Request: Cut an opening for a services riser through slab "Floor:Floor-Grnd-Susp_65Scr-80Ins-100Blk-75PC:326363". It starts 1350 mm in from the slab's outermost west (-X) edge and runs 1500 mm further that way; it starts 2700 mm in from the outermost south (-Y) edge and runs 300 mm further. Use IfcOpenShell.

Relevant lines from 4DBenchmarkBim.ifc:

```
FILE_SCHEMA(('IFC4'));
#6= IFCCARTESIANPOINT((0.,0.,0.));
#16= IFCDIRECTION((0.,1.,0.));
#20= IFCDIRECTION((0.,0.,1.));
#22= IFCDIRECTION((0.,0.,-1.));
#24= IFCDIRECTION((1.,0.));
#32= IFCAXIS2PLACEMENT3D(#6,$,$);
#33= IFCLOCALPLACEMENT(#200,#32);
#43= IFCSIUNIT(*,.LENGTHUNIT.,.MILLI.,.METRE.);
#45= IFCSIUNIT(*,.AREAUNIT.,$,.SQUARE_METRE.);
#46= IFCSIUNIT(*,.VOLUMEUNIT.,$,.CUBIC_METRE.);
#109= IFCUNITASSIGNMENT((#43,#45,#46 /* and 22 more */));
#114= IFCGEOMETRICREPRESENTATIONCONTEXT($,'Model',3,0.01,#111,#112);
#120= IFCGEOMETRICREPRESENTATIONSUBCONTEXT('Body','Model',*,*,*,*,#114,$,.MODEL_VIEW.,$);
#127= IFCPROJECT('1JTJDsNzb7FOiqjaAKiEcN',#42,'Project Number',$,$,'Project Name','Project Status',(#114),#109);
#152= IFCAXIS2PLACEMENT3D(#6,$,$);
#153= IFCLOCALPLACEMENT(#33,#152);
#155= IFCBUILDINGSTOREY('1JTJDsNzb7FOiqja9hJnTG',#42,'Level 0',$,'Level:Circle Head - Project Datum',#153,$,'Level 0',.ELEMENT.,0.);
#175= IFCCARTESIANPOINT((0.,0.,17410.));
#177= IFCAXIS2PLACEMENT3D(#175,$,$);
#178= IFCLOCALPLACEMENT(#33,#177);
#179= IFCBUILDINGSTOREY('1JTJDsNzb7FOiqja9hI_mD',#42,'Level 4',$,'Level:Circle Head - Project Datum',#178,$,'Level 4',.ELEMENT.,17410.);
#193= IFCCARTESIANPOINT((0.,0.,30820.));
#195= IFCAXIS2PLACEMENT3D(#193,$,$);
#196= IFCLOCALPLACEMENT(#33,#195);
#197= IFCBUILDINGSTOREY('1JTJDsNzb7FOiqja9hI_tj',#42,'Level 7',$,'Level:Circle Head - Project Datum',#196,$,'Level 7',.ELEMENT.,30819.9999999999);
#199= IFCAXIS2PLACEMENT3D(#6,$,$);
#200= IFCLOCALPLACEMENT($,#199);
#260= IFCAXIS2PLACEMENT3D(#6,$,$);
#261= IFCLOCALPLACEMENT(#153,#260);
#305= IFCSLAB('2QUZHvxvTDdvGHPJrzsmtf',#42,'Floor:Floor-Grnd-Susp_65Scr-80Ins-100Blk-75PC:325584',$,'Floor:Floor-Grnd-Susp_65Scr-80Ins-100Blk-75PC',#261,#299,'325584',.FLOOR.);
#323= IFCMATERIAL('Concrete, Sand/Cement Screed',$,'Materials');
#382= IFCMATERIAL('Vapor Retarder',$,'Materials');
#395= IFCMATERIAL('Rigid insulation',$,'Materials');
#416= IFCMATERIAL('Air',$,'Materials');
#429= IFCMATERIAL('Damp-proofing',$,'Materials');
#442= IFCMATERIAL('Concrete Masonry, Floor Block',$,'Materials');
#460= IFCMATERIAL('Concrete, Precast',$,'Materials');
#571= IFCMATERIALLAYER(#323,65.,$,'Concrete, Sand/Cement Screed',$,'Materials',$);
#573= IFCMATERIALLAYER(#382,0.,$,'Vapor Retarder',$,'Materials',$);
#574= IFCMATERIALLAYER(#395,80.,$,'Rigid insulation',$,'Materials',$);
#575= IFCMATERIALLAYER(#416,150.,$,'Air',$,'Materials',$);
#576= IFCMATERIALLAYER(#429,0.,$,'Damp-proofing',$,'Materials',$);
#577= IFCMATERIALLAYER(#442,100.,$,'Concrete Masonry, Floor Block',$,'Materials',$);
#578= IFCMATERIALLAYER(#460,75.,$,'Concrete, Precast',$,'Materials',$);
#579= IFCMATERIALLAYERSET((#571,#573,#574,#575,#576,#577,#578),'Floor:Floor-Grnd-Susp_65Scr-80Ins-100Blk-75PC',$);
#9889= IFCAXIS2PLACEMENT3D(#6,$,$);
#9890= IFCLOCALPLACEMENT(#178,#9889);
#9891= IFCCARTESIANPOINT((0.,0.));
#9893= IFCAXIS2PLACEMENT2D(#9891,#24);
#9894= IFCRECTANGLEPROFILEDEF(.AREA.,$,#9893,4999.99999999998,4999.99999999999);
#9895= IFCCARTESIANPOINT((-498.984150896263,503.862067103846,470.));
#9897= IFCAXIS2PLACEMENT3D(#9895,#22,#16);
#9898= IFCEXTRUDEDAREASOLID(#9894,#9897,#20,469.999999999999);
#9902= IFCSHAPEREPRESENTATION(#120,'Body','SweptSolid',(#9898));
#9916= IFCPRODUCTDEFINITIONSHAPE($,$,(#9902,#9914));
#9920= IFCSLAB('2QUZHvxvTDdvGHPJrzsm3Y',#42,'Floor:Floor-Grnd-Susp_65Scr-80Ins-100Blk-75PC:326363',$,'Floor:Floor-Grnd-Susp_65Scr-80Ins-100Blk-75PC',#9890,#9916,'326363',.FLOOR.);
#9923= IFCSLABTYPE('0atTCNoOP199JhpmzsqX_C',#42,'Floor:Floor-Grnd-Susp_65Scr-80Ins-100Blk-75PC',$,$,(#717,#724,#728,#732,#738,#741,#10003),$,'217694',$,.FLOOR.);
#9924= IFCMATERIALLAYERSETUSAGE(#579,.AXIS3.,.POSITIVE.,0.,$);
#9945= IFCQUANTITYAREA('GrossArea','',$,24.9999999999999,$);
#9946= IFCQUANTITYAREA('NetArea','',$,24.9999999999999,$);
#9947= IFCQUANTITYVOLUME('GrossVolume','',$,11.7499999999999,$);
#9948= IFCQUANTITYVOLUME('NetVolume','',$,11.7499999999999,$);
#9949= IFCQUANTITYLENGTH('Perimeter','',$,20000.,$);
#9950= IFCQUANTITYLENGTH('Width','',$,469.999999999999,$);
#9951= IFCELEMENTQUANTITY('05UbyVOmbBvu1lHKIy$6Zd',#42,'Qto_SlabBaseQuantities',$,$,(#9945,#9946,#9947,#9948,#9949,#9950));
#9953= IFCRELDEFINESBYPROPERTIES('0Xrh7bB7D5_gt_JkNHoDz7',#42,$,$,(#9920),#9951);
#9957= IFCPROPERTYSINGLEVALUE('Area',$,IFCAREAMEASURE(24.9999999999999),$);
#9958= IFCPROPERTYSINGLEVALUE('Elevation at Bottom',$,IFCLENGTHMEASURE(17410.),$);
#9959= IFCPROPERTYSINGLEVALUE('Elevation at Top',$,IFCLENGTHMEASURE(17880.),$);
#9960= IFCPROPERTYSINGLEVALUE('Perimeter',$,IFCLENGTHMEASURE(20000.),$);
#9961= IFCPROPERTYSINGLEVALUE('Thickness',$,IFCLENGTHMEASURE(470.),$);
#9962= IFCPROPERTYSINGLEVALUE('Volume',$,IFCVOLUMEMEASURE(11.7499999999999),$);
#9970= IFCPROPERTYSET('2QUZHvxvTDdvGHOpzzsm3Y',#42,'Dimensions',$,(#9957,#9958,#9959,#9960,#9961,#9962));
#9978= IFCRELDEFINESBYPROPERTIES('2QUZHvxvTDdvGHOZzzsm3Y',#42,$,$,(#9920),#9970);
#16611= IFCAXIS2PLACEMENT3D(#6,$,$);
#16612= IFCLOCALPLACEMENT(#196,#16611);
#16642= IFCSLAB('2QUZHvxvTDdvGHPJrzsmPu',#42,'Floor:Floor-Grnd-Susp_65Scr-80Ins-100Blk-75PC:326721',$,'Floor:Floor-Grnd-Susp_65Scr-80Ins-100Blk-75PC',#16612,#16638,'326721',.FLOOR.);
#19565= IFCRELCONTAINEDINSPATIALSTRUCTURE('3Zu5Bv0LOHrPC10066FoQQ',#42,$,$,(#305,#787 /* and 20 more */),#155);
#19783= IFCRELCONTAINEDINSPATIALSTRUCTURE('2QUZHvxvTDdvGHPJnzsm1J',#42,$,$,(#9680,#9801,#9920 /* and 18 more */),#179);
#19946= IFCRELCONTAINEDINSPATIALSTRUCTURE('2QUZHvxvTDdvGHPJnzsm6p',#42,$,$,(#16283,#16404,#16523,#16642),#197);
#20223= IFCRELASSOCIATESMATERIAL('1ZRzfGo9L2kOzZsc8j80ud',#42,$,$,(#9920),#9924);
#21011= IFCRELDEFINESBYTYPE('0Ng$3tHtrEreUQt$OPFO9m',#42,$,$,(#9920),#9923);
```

```python
import numpy as np
import ifcopenshell
import ifcopenshell.api.feature
import ifcopenshell.api.geometry
import ifcopenshell.api.pset
import ifcopenshell.api.root
import ifcopenshell.geom
import ifcopenshell.util.element
import ifcopenshell.util.placement
import ifcopenshell.util.representation
import ifcopenshell.util.shape
import ifcopenshell.util.unit

model = ifcopenshell.open("4DBenchmarkBim.ifc")
unit_scale = ifcopenshell.util.unit.calculate_unit_scale(model)
area_scale = ifcopenshell.util.unit.calculate_unit_scale(model, "AREAUNIT")
volume_scale = ifcopenshell.util.unit.calculate_unit_scale(model, "VOLUMEUNIT")
settings = ifcopenshell.geom.settings()


def volume(element):
    """Net volume in cubic metres, openings subtracted."""
    shape = ifcopenshell.geom.create_shape(settings, element)
    return ifcopenshell.util.shape.get_volume(shape.geometry)


slab = model.by_guid("2QUZHvxvTDdvGHPJrzsm3Y")
before = volume(slab)

# Extent in the slab's own axes, in metres. The edges named are its -X and -Y sides.
slab_shape = ifcopenshell.geom.create_shape(settings, slab)
vertices = ifcopenshell.util.shape.get_vertices(slab_shape.geometry)
x_min, y_min, bottom = vertices.min(axis=0)
top = vertices[:, 2].max()

opening = ifcopenshell.api.root.create_entity(model, ifc_class="IfcOpeningElement", name="Services riser opening", predefined_type="OPENING")
context = ifcopenshell.util.representation.get_context(model, "Model", "Body", "MODEL_VIEW")
width, depth = 1.5, 0.3
outline = [(0.0, 0.0), (width, 0.0), (width, depth), (0.0, depth), (0.0, 0.0)]
# Overshoot both faces by 50 mm so the cut is clean.
shape = ifcopenshell.api.geometry.add_slab_representation(
    model, context=context, depth=top - bottom + 0.1, polyline=outline
)
ifcopenshell.api.geometry.assign_representation(model, product=opening, representation=shape)

matrix = ifcopenshell.util.placement.get_local_placement(slab.ObjectPlacement)
matrix[:, 3] = matrix @ np.append(np.array([x_min + 1.35, y_min + 2.7, bottom - 0.05]) / unit_scale, 1.0)
ifcopenshell.api.geometry.edit_object_placement(model, product=opening, matrix=matrix, is_si=False)
ifcopenshell.api.feature.add_feature(model, feature=opening, element=slab)

after = volume(slab)

# Update the slab's stored quantities.
qto = model.by_id(ifcopenshell.util.element.get_pset(slab, "Qto_SlabBaseQuantities", should_inherit=False)["id"])
ifcopenshell.api.pset.edit_qto(model, qto=qto, properties={
    "NetArea": after / (top - bottom) / area_scale,
    "NetVolume": after / volume_scale,
})
pset = model.by_id(ifcopenshell.util.element.get_pset(slab, "Dimensions", should_inherit=False)["id"])
ifcopenshell.api.pset.edit_pset(model, pset=pset, properties={
    "Area": model.create_entity("IfcAreaMeasure", after / (top - bottom) / area_scale),
    "Volume": model.create_entity("IfcVolumeMeasure", after / volume_scale),
})

print(f"slab volume {before:.3f} -> {after:.3f} m3")

model.write("4DBenchmarkBim_v2.ifc")
```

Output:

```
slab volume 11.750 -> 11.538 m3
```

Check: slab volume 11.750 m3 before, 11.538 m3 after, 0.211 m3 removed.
